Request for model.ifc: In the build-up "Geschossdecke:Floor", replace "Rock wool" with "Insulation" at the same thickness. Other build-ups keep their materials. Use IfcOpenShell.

First a look at what the model holds.

```python
import ifcopenshell
import ifcopenshell.util.element

model = ifcopenshell.open("model.ifc")
print(model.schema)
for layer_set in model.by_type("IfcMaterialLayerSet"):
    if layer_set.LayerSetName == "Geschossdecke:Floor":
        for layer in layer_set.MaterialLayers:
            print(layer.id(), layer.Material and layer.Material.Name, layer.LayerThickness, sep=" | ")
        print(len(ifcopenshell.util.element.get_elements_by_material(model, layer_set)), "elements and types use it")
print(sorted(m.Name for m in model.by_type("IfcMaterial") if m.Name)[:60])
```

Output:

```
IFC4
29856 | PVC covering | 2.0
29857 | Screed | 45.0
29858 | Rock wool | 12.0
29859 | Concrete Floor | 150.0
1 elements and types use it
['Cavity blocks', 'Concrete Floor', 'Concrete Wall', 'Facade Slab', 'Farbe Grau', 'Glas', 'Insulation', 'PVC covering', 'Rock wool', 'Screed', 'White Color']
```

```python
import ifcopenshell
import ifcopenshell.api.material

model = ifcopenshell.open("model.ifc")

layer_set = next(s for s in model.by_type("IfcMaterialLayerSet") if s.LayerSetName == "Geschossdecke:Floor")
layer = next(l for l in layer_set.MaterialLayers if l.Material and l.Material.Name == "Rock wool")
material = next(m for m in model.by_type("IfcMaterial") if m.Name == "Insulation")

# Point this one layer at the other material; renaming the old one would change it everywhere.
ifcopenshell.api.material.edit_layer(model, layer=layer, attributes={}, material=material)

print([l.Material.Name if l.Material else None for l in layer_set.MaterialLayers])

model.write("model_v2.ifc")
```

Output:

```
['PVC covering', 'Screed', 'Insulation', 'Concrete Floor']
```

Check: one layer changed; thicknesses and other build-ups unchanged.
